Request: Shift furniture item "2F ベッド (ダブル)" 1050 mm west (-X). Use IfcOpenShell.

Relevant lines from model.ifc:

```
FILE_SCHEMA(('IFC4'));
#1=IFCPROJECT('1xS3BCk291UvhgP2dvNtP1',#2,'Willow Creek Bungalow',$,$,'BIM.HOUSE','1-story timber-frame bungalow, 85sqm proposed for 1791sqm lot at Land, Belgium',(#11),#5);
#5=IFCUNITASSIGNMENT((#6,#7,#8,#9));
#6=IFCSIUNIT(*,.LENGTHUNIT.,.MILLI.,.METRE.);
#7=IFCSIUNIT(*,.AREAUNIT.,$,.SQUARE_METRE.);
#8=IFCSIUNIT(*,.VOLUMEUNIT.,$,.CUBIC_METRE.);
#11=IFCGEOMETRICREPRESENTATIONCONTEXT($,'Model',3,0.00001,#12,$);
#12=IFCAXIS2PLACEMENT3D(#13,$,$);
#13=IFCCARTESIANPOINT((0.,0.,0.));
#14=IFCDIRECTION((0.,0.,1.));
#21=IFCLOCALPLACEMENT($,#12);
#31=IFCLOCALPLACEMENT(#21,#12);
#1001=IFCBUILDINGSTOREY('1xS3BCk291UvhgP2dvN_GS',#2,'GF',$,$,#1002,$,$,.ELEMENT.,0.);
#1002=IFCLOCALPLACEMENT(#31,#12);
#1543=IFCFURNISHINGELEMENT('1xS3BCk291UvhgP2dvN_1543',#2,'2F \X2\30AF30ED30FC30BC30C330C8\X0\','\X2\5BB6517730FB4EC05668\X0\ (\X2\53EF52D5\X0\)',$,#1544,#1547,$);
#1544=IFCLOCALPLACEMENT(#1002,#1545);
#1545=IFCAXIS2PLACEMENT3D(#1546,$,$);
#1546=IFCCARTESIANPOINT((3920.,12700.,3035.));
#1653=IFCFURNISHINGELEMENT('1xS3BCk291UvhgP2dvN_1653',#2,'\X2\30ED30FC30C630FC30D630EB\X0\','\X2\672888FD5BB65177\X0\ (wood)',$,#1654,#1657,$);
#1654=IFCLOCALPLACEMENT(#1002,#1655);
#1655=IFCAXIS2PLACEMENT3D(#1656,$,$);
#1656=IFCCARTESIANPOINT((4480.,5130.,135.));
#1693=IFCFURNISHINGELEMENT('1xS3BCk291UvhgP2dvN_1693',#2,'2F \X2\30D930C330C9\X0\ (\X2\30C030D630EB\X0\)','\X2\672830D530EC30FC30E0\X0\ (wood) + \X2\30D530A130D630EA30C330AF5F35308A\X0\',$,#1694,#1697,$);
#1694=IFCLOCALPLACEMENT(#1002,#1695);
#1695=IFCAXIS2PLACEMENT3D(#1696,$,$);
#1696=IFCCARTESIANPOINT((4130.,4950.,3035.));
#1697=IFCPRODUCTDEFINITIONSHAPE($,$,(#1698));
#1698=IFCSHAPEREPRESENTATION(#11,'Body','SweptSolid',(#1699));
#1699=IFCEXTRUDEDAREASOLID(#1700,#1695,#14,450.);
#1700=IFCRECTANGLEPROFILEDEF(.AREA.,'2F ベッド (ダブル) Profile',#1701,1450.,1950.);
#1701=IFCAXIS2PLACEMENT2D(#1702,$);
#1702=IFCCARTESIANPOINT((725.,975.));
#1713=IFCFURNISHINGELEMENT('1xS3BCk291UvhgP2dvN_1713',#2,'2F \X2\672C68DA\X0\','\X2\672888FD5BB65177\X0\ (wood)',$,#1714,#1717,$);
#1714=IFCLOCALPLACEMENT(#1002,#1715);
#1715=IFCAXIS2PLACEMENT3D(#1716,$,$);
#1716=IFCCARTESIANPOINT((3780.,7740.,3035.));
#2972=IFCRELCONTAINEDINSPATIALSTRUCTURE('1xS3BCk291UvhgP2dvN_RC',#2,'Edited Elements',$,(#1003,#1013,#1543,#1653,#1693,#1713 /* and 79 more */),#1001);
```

```python
import ifcopenshell
import ifcopenshell.api.geometry
import ifcopenshell.util.placement
import ifcopenshell.util.unit

model = ifcopenshell.open("model.ifc")
unit_scale = ifcopenshell.util.unit.calculate_unit_scale(model)

item = model.by_id(1693)
matrix = ifcopenshell.util.placement.get_local_placement(item.ObjectPlacement)
matrix[0, 3] -= 1.05 / unit_scale
ifcopenshell.api.geometry.edit_object_placement(model, product=item, matrix=matrix, is_si=False)

print(ifcopenshell.util.placement.get_local_placement(item.ObjectPlacement).round(3) + 0.0)

model.write("model_rev.ifc")
```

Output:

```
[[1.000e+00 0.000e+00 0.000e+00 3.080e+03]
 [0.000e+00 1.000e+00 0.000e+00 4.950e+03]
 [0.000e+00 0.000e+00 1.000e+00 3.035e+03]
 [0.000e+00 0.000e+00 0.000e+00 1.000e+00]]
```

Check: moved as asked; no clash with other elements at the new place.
